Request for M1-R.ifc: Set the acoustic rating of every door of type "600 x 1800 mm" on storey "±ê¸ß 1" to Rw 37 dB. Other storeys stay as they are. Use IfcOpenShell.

First a look at what the model holds.

```python
import ifcopenshell
import ifcopenshell.util.element

model = ifcopenshell.open("M1-R.ifc")
print(model.schema)
storey = next(s for s in model.by_type("IfcBuildingStorey") if s.Name == "±ê¸ß 1")
doors = [e for e in ifcopenshell.util.element.get_decomposition(storey) if e.is_a("IfcDoor")]
seen = {}
for e in doors:
    element_type = ifcopenshell.util.element.get_type(e)
    key = (element_type.Name if element_type != e and element_type else None, ifcopenshell.util.element.get_pset(e, "Pset_DoorCommon", "AcousticRating"))
    seen[key] = seen.get(key, 0) + 1
for (name, value), count in sorted(seen.items(), key=str):
    print(count, "x", name, "|", value)
```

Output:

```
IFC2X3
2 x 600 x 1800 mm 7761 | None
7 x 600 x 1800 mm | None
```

```python
import ifcopenshell
import ifcopenshell.api.pset
import ifcopenshell.util.element

model = ifcopenshell.open("M1-R.ifc")

storey = next(s for s in model.by_type("IfcBuildingStorey") if s.Name == "±ê¸ß 1")
doors = [e for e in ifcopenshell.util.element.get_decomposition(storey) if e.is_a("IfcDoor")]

count = 0
for e in doors:
    element_type = ifcopenshell.util.element.get_type(e)
    if element_type in (None, e) or element_type.Name != "600 x 1800 mm":
        continue
    # add_pset returns the element's existing set when there is one.
    pset = ifcopenshell.api.pset.add_pset(model, product=e, name="Pset_DoorCommon")
    ifcopenshell.api.pset.edit_pset(model, pset=pset, properties={"AcousticRating": "Rw 37 dB"})
    count += 1

print(count, "doors updated")

model.write("M1-R_v2.ifc")
```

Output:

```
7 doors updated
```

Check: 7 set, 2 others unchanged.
